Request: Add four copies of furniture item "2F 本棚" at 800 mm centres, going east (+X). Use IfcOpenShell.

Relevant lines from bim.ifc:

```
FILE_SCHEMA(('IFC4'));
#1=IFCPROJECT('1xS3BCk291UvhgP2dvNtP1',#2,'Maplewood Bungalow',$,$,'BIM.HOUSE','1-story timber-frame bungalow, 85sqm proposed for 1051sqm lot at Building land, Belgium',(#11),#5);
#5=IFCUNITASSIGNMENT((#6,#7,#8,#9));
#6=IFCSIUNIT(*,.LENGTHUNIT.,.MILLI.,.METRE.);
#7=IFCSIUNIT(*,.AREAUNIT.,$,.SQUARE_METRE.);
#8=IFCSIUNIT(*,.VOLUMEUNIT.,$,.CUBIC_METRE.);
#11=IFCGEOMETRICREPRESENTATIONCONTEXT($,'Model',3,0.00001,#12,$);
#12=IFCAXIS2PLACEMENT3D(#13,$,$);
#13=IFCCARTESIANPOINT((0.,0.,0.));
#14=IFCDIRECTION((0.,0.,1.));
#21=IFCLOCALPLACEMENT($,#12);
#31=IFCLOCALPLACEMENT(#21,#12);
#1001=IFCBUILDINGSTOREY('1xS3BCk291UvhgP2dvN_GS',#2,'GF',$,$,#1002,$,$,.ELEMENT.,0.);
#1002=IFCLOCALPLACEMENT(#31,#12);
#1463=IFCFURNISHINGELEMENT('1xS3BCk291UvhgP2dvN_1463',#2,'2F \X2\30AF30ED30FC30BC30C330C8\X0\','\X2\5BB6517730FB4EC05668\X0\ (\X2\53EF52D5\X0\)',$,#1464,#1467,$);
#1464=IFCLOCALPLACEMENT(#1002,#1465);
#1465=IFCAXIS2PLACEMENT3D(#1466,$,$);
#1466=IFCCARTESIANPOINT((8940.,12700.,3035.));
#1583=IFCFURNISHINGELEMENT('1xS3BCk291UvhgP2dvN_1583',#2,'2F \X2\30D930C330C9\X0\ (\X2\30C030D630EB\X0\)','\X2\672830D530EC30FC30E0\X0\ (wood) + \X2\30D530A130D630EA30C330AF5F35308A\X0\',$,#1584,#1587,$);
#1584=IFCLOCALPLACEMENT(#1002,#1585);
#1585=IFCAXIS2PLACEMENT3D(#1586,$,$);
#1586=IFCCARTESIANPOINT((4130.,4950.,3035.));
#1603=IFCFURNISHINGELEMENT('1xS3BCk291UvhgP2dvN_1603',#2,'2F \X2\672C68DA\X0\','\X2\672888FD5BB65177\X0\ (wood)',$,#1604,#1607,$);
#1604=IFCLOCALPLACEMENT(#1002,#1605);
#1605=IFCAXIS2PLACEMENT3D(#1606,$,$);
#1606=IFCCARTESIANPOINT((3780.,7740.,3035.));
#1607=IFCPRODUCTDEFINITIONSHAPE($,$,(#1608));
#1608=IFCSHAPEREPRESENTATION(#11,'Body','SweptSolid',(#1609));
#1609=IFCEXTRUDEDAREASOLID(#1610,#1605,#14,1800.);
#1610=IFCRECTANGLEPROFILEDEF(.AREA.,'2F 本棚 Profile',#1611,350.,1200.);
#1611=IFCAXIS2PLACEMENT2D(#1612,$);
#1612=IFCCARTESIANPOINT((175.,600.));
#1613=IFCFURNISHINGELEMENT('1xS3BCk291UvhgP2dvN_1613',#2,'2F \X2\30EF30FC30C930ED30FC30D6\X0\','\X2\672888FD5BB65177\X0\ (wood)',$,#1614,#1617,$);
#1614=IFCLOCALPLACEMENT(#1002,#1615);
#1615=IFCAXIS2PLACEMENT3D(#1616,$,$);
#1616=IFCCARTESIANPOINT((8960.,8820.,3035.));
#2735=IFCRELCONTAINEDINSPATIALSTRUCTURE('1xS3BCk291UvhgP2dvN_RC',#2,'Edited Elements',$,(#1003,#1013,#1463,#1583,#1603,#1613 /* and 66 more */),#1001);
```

```python
import numpy as np
import ifcopenshell
import ifcopenshell.api.geometry
import ifcopenshell.api.root
import ifcopenshell.util.element
import ifcopenshell.util.placement
import ifcopenshell.util.unit

model = ifcopenshell.open("bim.ifc")
unit_scale = ifcopenshell.util.unit.calculate_unit_scale(model)


def reuse_history(source, copy):
    """copy_class also copies each property set's owner history, people and application; keep the originals."""
    for rel in copy.IsDefinedBy:
        if rel.is_a("IfcRelDefinesByProperties") and (history := rel.RelatingPropertyDefinition.OwnerHistory):
            rel.RelatingPropertyDefinition.OwnerHistory = source.OwnerHistory
            ifcopenshell.util.element.remove_deep2(model, history)


source = model.by_guid("1xS3BCk291UvhgP2dvN_1603")
base = ifcopenshell.util.placement.get_local_placement(source.ObjectPlacement)
step = np.array([1.0, 0.0, 0.0]) * 0.8 / unit_scale

for i in range(1, 5):
    copy = ifcopenshell.api.root.copy_class(model, product=source)
    copy.Representation = ifcopenshell.util.element.copy_deep(
        model, source.Representation, exclude=["IfcGeometricRepresentationContext", "IfcRepresentationMap"]
    )
    reuse_history(source, copy)
    matrix = base.copy()
    matrix[:3, 3] += i * step
    print("added at", matrix[:3, 3].round(3) + 0.0)
    ifcopenshell.api.geometry.edit_object_placement(model, product=copy, matrix=matrix, is_si=False)

model.write("bim_rev.ifc")
```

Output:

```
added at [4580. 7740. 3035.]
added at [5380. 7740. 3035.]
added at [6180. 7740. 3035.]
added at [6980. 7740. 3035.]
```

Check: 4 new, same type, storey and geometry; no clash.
